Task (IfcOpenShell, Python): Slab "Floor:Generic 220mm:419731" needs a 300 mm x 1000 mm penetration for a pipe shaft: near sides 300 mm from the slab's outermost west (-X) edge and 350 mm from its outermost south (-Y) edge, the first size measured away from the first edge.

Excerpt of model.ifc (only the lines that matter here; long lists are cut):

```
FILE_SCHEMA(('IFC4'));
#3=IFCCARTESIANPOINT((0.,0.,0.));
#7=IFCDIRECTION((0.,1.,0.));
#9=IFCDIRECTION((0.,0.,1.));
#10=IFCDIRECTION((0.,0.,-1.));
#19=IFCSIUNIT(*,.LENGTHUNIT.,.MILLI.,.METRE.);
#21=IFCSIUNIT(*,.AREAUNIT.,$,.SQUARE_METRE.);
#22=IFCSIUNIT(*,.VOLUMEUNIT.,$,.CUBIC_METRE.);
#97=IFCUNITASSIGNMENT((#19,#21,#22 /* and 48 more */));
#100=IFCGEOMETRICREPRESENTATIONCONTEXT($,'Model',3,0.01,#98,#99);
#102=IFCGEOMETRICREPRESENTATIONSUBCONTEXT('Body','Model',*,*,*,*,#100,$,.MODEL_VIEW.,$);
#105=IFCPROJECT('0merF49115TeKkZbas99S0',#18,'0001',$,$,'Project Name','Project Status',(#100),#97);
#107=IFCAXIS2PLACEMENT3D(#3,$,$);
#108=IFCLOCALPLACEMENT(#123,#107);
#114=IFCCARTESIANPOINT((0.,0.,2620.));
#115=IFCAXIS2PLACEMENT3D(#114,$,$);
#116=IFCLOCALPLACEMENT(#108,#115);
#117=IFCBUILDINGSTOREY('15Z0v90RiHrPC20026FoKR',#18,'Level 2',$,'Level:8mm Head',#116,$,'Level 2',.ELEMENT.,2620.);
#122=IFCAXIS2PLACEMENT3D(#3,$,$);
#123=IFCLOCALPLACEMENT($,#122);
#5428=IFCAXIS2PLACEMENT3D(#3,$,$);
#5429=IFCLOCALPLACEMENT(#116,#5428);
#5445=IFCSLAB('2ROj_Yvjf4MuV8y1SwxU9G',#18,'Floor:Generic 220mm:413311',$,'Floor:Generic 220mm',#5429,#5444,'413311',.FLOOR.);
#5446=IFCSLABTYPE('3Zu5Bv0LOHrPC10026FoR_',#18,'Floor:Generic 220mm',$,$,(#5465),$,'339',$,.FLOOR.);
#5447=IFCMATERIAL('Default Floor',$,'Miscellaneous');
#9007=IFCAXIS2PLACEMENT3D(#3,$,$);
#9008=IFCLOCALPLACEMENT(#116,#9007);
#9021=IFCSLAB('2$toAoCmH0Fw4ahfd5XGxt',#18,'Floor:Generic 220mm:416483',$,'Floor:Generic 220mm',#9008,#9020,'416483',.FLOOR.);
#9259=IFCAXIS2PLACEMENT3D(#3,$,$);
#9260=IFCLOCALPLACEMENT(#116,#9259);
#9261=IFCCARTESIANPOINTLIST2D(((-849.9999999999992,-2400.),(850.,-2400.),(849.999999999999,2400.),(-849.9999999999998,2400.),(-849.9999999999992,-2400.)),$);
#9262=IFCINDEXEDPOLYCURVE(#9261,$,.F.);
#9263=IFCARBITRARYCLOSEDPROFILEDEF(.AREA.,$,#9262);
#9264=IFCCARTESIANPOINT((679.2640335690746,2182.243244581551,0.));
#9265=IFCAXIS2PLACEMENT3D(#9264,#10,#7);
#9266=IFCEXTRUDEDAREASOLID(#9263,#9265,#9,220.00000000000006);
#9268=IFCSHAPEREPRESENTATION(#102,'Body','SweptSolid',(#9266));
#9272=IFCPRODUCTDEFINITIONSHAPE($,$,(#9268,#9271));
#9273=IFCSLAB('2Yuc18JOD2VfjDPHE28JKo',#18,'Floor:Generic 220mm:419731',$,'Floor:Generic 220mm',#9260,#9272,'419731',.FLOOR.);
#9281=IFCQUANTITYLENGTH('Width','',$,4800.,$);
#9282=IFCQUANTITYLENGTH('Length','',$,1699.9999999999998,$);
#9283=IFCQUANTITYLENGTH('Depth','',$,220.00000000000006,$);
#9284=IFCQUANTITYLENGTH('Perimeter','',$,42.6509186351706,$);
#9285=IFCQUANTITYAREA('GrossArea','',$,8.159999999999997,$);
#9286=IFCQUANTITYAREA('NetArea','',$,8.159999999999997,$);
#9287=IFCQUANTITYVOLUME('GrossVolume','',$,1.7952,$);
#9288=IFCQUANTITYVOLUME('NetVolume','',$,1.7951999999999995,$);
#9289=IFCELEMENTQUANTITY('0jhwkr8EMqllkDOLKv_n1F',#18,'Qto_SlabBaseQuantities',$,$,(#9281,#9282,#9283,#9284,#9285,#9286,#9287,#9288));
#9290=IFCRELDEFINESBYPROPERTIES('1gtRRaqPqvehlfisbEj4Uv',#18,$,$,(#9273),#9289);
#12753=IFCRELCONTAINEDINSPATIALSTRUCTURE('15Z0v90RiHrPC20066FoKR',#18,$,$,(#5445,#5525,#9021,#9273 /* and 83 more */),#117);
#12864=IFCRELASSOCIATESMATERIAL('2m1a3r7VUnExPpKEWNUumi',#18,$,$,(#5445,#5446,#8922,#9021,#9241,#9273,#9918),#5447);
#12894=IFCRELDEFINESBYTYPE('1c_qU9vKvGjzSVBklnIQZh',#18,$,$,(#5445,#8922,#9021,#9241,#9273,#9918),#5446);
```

```python
import numpy as np
import ifcopenshell
import ifcopenshell.api.feature
import ifcopenshell.api.geometry
import ifcopenshell.api.pset
import ifcopenshell.api.root
import ifcopenshell.geom
import ifcopenshell.util.element
import ifcopenshell.util.placement
import ifcopenshell.util.representation
import ifcopenshell.util.shape
import ifcopenshell.util.unit

model = ifcopenshell.open("model.ifc")
unit_scale = ifcopenshell.util.unit.calculate_unit_scale(model)
area_scale = ifcopenshell.util.unit.calculate_unit_scale(model, "AREAUNIT")
volume_scale = ifcopenshell.util.unit.calculate_unit_scale(model, "VOLUMEUNIT")
settings = ifcopenshell.geom.settings()


def volume(element):
    """Net volume in cubic metres, openings subtracted."""
    shape = ifcopenshell.geom.create_shape(settings, element)
    return ifcopenshell.util.shape.get_volume(shape.geometry)


slab = model.by_guid("2Yuc18JOD2VfjDPHE28JKo")
before = volume(slab)

# Extent in the slab's own axes, in metres. The edges named are its -X and -Y sides.
slab_shape = ifcopenshell.geom.create_shape(settings, slab)
vertices = ifcopenshell.util.shape.get_vertices(slab_shape.geometry)
x_min, y_min, bottom = vertices.min(axis=0)
top = vertices[:, 2].max()

opening = ifcopenshell.api.root.create_entity(model, ifc_class="IfcOpeningElement", name="Pipe shaft opening", predefined_type="OPENING")
context = ifcopenshell.util.representation.get_context(model, "Model", "Body", "MODEL_VIEW")
width, depth = 0.3, 1
outline = [(0.0, 0.0), (width, 0.0), (width, depth), (0.0, depth), (0.0, 0.0)]
# Overshoot both faces by 50 mm so the cut is clean.
shape = ifcopenshell.api.geometry.add_slab_representation(
    model, context=context, depth=top - bottom + 0.1, polyline=outline
)
ifcopenshell.api.geometry.assign_representation(model, product=opening, representation=shape)

matrix = ifcopenshell.util.placement.get_local_placement(slab.ObjectPlacement)
matrix[:, 3] = matrix @ np.append(np.array([x_min + 0.3, y_min + 0.35, bottom - 0.05]) / unit_scale, 1.0)
ifcopenshell.api.geometry.edit_object_placement(model, product=opening, matrix=matrix, is_si=False)
ifcopenshell.api.feature.add_feature(model, feature=opening, element=slab)

after = volume(slab)

# Update the slab's stored quantities.
qto = model.by_id(ifcopenshell.util.element.get_pset(slab, "Qto_SlabBaseQuantities", should_inherit=False)["id"])
ifcopenshell.api.pset.edit_qto(model, qto=qto, properties={
    "NetArea": after / (top - bottom) / area_scale,
    "NetVolume": after / volume_scale,
})

print(f"slab volume {before:.3f} -> {after:.3f} m3")

model.write("model_rev.ifc")
```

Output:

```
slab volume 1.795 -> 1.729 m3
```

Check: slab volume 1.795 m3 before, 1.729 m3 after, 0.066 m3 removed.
